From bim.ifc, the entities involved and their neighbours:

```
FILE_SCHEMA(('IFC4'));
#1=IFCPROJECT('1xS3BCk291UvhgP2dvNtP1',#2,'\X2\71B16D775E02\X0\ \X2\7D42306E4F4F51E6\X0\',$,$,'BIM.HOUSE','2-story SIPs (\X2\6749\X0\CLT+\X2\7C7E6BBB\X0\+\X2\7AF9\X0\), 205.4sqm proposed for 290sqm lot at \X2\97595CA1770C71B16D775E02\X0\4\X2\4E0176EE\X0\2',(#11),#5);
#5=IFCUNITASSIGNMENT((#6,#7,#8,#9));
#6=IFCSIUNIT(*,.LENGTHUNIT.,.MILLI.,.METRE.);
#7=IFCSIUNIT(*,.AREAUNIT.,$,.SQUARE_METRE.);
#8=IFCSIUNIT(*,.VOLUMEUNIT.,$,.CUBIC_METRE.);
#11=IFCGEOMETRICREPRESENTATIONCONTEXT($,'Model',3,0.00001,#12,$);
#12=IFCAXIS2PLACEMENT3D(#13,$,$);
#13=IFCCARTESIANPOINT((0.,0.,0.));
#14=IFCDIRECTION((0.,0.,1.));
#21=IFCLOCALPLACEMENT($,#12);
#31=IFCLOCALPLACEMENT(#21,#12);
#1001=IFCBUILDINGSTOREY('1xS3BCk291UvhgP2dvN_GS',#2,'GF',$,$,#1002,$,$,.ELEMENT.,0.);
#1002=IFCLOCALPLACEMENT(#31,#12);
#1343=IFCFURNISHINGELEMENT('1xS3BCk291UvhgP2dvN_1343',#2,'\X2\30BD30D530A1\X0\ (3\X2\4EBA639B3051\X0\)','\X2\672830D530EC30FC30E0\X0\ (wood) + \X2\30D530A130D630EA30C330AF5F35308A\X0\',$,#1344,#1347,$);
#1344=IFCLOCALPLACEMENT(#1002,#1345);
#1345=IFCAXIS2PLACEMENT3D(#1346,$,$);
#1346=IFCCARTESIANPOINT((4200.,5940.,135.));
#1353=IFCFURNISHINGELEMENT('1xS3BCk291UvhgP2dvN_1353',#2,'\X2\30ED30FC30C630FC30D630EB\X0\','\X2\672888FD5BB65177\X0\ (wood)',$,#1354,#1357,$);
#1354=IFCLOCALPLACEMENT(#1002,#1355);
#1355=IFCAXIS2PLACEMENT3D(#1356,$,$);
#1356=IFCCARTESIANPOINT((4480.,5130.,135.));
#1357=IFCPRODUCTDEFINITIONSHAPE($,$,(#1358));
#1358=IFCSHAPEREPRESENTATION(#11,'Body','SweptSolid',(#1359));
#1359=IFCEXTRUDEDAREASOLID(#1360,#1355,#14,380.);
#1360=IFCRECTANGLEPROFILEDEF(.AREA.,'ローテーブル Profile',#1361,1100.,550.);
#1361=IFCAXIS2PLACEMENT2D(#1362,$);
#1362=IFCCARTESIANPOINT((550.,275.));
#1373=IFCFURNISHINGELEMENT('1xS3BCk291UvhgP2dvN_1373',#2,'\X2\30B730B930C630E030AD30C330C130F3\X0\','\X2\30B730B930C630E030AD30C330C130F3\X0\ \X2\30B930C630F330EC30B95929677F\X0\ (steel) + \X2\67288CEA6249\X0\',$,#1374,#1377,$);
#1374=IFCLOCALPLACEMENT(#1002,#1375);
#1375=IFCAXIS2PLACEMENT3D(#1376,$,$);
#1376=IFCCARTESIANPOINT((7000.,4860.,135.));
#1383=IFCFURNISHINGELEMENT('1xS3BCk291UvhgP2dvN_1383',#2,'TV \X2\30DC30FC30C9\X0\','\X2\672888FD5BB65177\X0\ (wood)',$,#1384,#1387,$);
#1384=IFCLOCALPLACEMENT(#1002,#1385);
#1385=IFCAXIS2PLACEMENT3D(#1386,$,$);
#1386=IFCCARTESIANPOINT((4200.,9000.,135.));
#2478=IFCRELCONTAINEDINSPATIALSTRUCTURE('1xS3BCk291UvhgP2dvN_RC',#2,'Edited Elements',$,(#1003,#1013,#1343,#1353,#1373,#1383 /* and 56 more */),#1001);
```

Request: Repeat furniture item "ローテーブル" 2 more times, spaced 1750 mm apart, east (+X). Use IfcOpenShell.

```python
import numpy as np
import ifcopenshell
import ifcopenshell.api.geometry
import ifcopenshell.api.root
import ifcopenshell.util.element
import ifcopenshell.util.placement

model = ifcopenshell.open("bim.ifc")


def reuse_history(source, copy):
    """copy_class also copies each property set's owner history, people and application; keep the originals."""
    for rel in copy.IsDefinedBy:
        if rel.is_a("IfcRelDefinesByProperties") and (history := rel.RelatingPropertyDefinition.OwnerHistory):
            rel.RelatingPropertyDefinition.OwnerHistory = source.OwnerHistory
            ifcopenshell.util.element.remove_deep2(model, history)


source = model.by_guid("1xS3BCk291UvhgP2dvN_1353")
base = ifcopenshell.util.placement.get_local_placement(source.ObjectPlacement)
step = np.array([1.0, 0.0, 0.0]) * 1750.0

for i in range(1, 3):
    copy = ifcopenshell.api.root.copy_class(model, product=source)
    copy.Representation = ifcopenshell.util.element.copy_deep(
        model, source.Representation, exclude=["IfcGeometricRepresentationContext", "IfcRepresentationMap"]
    )
    reuse_history(source, copy)
    matrix = base.copy()
    matrix[:3, 3] += i * step
    print("added at", matrix[:3, 3].round(3) + 0.0)
    ifcopenshell.api.geometry.edit_object_placement(model, product=copy, matrix=matrix, is_si=False)

model.write("bim_updated.ifc")
```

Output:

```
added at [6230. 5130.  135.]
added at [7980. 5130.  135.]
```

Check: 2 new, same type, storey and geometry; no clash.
